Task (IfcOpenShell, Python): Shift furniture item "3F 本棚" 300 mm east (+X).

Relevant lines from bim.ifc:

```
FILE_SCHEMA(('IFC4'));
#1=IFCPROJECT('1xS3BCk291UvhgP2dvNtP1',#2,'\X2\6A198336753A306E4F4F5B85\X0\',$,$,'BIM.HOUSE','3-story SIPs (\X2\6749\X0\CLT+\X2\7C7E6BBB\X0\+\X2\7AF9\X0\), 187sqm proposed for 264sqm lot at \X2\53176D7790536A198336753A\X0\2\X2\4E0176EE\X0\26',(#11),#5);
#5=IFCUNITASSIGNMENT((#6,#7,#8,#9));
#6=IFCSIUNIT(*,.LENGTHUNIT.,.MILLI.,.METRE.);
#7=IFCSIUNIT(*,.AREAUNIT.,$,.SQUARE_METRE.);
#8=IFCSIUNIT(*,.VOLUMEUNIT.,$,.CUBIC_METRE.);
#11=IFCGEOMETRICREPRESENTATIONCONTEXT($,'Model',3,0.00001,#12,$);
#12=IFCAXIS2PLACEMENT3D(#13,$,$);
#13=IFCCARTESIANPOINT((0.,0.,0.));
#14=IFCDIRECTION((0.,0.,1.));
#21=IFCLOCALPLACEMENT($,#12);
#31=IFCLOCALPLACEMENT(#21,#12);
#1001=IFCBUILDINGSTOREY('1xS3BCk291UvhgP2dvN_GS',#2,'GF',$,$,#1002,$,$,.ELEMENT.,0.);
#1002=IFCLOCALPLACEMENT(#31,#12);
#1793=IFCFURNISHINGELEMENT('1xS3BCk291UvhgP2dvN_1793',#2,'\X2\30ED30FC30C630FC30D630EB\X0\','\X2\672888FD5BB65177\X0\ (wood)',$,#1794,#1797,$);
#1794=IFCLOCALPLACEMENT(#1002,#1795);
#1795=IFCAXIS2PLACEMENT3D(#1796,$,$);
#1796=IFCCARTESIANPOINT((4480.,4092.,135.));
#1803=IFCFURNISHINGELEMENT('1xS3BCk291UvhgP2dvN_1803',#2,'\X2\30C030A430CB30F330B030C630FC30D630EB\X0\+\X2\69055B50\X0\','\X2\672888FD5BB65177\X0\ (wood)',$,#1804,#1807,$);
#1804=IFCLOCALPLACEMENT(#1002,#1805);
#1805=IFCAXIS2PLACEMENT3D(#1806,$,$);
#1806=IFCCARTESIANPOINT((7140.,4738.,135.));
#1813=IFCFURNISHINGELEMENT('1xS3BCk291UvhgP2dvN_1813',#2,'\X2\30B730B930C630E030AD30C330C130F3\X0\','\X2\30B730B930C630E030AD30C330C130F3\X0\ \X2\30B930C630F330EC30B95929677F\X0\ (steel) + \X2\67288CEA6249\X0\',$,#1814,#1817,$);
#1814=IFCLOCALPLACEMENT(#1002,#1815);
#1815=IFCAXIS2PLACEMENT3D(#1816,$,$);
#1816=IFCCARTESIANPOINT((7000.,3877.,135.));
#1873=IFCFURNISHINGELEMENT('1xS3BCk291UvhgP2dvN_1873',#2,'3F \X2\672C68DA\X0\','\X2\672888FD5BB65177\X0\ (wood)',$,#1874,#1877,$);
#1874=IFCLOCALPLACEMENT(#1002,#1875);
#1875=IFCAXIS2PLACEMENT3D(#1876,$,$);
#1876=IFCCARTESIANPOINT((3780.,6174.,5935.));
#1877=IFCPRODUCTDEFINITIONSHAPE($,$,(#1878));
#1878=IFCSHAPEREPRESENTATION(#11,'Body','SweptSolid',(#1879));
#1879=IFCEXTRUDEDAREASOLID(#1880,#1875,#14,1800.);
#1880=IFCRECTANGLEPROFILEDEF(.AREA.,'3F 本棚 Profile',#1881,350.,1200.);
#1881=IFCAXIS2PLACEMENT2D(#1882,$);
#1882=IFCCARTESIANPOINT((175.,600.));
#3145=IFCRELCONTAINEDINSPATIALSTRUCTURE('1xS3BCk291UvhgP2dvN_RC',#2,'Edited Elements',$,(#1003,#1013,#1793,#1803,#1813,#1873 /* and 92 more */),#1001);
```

```python
import ifcopenshell
import ifcopenshell.api.geometry
import ifcopenshell.util.placement
import ifcopenshell.util.unit

model = ifcopenshell.open("bim.ifc")
unit_scale = ifcopenshell.util.unit.calculate_unit_scale(model)

item = model.by_guid("1xS3BCk291UvhgP2dvN_1873")
matrix = ifcopenshell.util.placement.get_local_placement(item.ObjectPlacement)
matrix[0, 3] += 0.3 / unit_scale
ifcopenshell.api.geometry.edit_object_placement(model, product=item, matrix=matrix, is_si=False)

print(ifcopenshell.util.placement.get_local_placement(item.ObjectPlacement).round(3) + 0.0)

model.write("bim_edited.ifc")
```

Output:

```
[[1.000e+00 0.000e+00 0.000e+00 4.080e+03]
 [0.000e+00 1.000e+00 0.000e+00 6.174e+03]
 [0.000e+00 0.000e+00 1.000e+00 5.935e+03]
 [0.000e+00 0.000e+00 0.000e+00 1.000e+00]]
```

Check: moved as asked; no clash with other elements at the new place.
